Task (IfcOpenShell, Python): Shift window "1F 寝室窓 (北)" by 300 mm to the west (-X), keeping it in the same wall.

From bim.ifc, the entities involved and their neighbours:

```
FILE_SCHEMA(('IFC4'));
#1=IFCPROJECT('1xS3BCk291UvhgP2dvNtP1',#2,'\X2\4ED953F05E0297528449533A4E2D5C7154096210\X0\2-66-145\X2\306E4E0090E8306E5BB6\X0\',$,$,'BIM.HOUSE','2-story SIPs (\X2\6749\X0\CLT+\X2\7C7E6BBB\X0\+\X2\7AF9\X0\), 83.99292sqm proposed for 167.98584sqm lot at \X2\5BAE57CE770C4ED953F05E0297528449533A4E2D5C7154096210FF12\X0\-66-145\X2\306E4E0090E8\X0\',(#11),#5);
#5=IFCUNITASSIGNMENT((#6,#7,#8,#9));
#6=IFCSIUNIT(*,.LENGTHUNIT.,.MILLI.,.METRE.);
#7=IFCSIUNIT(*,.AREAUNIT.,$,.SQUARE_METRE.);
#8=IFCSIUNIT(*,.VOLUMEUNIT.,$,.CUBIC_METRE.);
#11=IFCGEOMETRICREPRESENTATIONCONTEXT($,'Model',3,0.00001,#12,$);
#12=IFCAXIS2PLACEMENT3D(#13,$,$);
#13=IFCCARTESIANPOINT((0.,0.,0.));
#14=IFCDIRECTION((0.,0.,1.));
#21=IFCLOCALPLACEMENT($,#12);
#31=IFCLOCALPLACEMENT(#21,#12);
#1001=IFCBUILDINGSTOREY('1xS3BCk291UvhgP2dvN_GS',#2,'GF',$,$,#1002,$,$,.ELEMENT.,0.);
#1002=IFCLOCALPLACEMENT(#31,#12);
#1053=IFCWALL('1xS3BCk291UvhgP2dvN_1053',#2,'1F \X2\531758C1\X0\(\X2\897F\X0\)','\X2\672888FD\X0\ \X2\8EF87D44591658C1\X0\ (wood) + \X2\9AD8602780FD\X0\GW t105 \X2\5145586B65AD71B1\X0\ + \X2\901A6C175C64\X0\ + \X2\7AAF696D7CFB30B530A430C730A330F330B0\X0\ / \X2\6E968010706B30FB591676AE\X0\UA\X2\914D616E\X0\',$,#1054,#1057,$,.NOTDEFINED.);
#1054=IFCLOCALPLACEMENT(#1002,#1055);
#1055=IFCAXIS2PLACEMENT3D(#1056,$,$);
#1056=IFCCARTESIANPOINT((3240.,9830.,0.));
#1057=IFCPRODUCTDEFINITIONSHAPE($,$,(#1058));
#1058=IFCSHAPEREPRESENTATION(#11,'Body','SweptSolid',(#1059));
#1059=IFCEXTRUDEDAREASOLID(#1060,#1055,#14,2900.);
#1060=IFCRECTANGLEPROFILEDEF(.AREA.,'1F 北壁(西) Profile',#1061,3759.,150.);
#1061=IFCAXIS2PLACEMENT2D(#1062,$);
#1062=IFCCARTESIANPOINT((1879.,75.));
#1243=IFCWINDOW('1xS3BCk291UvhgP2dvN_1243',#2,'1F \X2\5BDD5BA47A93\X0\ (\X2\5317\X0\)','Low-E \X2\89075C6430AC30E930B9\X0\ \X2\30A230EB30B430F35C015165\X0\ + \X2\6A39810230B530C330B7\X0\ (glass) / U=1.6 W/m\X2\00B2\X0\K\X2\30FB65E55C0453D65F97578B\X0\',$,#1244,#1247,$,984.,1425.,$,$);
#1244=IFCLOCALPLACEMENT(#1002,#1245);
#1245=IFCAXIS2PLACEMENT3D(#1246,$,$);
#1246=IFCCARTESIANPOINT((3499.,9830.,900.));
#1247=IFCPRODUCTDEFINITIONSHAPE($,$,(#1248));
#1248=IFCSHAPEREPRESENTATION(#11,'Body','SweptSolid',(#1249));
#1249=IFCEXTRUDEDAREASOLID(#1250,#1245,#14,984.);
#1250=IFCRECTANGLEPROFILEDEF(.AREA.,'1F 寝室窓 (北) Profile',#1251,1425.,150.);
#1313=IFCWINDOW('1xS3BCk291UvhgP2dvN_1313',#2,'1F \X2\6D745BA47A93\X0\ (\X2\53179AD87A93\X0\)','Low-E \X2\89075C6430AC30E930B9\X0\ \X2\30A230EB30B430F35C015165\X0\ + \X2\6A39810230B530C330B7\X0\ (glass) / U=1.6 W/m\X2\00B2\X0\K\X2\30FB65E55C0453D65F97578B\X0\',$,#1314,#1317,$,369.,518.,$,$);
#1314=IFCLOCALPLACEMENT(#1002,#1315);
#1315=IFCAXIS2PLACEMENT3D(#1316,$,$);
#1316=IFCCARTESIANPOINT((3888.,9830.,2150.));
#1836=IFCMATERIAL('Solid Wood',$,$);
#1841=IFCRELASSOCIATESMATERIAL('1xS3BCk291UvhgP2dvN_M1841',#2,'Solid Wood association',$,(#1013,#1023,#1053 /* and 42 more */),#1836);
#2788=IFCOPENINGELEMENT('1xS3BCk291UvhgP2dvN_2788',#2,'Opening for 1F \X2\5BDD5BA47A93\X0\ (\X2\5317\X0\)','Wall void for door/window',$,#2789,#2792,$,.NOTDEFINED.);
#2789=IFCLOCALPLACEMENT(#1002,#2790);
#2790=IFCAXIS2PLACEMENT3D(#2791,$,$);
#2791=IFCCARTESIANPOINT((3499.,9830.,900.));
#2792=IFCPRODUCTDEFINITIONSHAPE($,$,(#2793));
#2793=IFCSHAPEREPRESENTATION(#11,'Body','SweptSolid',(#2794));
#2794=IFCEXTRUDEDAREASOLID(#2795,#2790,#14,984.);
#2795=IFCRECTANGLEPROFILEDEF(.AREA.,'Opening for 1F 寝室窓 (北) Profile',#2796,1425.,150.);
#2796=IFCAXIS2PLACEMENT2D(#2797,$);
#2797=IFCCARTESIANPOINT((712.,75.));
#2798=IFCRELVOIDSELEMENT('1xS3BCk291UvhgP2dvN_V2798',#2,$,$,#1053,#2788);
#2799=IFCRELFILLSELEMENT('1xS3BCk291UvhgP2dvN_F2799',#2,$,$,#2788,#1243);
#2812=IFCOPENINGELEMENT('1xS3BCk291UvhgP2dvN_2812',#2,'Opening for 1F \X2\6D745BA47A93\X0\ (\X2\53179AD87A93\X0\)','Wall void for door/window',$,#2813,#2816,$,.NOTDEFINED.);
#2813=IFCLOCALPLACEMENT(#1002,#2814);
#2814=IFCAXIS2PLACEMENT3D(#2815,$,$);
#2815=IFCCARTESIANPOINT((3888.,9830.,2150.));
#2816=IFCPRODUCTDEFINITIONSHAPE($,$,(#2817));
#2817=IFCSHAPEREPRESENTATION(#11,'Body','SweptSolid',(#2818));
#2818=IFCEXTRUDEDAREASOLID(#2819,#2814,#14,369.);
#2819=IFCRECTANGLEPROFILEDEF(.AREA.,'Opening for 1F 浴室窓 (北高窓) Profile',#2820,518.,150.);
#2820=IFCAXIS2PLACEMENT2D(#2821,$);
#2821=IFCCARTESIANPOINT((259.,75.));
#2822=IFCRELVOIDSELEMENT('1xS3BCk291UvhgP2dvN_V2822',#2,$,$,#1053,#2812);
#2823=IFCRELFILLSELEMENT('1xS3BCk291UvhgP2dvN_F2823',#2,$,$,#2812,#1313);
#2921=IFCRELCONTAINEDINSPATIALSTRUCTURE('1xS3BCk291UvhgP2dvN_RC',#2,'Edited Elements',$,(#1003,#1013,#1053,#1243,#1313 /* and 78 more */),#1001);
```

```python
import ifcopenshell
import ifcopenshell.api.geometry
import ifcopenshell.util.placement

model = ifcopenshell.open("bim.ifc")

window = model.by_guid("1xS3BCk291UvhgP2dvN_1243")
opening = window.FillsVoids[0].RelatingOpeningElement
wall = opening.VoidsElements[0].RelatingBuildingElement

wall_matrix = ifcopenshell.util.placement.get_local_placement(wall.ObjectPlacement)
shift = wall_matrix[:3, 0] * -300.0
before = ifcopenshell.util.placement.get_local_placement(window.ObjectPlacement)[:3, 3].copy()

# The window is not placed relative to its opening, so move both.
for product in (opening, window):
    matrix = ifcopenshell.util.placement.get_local_placement(product.ObjectPlacement)
    matrix[:3, 3] += shift
    ifcopenshell.api.geometry.edit_object_placement(model, product=product, matrix=matrix, is_si=False)

after = ifcopenshell.util.placement.get_local_placement(window.ObjectPlacement)[:3, 3]
print("window moved by", (after - before).round(3) + 0.0)

model.write("bim-out.ifc")
```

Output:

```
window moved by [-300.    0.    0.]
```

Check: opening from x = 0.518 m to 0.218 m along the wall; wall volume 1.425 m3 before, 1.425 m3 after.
